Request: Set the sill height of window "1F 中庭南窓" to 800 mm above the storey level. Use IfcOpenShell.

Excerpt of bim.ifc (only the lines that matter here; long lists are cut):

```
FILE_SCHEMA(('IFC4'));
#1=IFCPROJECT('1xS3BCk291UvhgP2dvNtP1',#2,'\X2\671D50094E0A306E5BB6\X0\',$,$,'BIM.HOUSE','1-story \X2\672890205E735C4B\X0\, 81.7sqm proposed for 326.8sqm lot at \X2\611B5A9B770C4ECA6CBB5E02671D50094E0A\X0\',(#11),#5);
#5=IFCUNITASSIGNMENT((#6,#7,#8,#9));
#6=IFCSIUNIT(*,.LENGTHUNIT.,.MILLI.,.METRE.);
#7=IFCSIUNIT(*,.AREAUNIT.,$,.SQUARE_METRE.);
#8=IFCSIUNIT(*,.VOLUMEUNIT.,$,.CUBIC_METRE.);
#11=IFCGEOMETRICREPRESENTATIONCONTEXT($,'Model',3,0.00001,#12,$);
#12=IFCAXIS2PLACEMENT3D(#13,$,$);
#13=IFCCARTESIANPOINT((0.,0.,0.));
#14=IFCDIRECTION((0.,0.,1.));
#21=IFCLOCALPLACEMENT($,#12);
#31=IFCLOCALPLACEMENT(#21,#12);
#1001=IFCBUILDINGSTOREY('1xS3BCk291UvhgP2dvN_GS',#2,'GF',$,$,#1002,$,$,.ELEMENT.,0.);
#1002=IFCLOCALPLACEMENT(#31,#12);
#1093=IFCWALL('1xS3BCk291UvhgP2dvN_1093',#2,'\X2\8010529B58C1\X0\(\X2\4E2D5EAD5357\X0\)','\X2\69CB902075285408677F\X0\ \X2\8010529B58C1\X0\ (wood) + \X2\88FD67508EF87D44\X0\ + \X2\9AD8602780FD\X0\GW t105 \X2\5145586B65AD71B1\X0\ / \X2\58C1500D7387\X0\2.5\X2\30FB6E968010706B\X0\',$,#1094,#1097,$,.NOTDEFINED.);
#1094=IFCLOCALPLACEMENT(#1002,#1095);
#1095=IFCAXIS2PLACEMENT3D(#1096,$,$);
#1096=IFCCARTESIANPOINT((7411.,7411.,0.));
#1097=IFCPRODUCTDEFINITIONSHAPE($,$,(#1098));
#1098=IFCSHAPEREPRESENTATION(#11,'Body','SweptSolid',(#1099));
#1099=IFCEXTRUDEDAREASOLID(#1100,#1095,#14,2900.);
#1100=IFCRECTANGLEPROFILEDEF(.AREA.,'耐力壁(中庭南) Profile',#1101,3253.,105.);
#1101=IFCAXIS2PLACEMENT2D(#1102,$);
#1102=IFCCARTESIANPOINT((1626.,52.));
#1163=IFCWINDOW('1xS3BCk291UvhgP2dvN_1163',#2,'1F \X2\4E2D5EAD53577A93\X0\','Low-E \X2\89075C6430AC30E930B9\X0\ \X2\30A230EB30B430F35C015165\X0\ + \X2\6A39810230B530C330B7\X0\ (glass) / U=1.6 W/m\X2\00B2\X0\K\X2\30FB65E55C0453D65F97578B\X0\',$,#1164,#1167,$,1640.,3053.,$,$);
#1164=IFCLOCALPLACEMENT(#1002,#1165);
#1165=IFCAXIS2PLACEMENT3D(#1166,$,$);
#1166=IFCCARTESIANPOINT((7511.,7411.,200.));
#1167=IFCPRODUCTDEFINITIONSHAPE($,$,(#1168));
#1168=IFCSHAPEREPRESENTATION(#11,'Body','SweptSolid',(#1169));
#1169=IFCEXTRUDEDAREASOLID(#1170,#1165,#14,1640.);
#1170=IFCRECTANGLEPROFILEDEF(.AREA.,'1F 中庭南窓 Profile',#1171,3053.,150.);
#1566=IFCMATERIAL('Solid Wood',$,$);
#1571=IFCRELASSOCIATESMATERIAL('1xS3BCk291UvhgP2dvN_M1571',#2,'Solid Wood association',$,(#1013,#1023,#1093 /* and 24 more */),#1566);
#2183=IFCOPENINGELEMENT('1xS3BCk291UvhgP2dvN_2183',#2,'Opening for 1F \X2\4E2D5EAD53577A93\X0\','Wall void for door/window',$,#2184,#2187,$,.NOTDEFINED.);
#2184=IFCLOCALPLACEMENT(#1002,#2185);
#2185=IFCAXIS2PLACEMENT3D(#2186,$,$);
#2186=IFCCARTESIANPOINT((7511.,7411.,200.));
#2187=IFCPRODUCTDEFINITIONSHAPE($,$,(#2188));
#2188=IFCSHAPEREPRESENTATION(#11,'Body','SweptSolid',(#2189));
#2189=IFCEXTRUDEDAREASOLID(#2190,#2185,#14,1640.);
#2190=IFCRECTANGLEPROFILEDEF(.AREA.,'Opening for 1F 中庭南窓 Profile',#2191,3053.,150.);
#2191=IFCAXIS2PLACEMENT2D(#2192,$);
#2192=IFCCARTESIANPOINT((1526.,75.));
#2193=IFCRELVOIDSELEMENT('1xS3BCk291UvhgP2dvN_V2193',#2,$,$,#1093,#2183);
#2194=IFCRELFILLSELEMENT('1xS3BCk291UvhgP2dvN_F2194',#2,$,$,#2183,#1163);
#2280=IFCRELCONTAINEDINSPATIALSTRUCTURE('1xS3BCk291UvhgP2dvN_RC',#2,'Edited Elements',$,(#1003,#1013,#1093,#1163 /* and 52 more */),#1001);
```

```python
import numpy as np
import ifcopenshell
import ifcopenshell.api.geometry
import ifcopenshell.geom
import ifcopenshell.util.element
import ifcopenshell.util.placement
import ifcopenshell.util.shape
import ifcopenshell.util.unit

model = ifcopenshell.open("bim.ifc")
unit_scale = ifcopenshell.util.unit.calculate_unit_scale(model)

window = model.by_guid("1xS3BCk291UvhgP2dvN_1163")
opening = window.FillsVoids[0].RelatingOpeningElement
storey = ifcopenshell.util.element.get_container(window, ifc_class="IfcBuildingStorey")
level = ifcopenshell.util.placement.get_local_placement(storey.ObjectPlacement)[2, 3]

# The opening's origin need not be at the sill, so measure its lowest point.
shape = ifcopenshell.geom.create_shape(ifcopenshell.geom.settings(), opening)
bottom = ifcopenshell.util.shape.get_shape_bottom_elevation(shape, shape.geometry) / unit_scale
dz = level + 800.0 - bottom

shift = np.array([0.0, 0.0, dz])
# The window is not placed relative to its opening, so move both.
for product in (opening, window):
    matrix = ifcopenshell.util.placement.get_local_placement(product.ObjectPlacement)
    matrix[:3, 3] += shift
    ifcopenshell.api.geometry.edit_object_placement(model, product=product, matrix=matrix, is_si=False)

print(f"moved by {dz * unit_scale:+.3f} m")

model.write("bim_rev.ifc")
```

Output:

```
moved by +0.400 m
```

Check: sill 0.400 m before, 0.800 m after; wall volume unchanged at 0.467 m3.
